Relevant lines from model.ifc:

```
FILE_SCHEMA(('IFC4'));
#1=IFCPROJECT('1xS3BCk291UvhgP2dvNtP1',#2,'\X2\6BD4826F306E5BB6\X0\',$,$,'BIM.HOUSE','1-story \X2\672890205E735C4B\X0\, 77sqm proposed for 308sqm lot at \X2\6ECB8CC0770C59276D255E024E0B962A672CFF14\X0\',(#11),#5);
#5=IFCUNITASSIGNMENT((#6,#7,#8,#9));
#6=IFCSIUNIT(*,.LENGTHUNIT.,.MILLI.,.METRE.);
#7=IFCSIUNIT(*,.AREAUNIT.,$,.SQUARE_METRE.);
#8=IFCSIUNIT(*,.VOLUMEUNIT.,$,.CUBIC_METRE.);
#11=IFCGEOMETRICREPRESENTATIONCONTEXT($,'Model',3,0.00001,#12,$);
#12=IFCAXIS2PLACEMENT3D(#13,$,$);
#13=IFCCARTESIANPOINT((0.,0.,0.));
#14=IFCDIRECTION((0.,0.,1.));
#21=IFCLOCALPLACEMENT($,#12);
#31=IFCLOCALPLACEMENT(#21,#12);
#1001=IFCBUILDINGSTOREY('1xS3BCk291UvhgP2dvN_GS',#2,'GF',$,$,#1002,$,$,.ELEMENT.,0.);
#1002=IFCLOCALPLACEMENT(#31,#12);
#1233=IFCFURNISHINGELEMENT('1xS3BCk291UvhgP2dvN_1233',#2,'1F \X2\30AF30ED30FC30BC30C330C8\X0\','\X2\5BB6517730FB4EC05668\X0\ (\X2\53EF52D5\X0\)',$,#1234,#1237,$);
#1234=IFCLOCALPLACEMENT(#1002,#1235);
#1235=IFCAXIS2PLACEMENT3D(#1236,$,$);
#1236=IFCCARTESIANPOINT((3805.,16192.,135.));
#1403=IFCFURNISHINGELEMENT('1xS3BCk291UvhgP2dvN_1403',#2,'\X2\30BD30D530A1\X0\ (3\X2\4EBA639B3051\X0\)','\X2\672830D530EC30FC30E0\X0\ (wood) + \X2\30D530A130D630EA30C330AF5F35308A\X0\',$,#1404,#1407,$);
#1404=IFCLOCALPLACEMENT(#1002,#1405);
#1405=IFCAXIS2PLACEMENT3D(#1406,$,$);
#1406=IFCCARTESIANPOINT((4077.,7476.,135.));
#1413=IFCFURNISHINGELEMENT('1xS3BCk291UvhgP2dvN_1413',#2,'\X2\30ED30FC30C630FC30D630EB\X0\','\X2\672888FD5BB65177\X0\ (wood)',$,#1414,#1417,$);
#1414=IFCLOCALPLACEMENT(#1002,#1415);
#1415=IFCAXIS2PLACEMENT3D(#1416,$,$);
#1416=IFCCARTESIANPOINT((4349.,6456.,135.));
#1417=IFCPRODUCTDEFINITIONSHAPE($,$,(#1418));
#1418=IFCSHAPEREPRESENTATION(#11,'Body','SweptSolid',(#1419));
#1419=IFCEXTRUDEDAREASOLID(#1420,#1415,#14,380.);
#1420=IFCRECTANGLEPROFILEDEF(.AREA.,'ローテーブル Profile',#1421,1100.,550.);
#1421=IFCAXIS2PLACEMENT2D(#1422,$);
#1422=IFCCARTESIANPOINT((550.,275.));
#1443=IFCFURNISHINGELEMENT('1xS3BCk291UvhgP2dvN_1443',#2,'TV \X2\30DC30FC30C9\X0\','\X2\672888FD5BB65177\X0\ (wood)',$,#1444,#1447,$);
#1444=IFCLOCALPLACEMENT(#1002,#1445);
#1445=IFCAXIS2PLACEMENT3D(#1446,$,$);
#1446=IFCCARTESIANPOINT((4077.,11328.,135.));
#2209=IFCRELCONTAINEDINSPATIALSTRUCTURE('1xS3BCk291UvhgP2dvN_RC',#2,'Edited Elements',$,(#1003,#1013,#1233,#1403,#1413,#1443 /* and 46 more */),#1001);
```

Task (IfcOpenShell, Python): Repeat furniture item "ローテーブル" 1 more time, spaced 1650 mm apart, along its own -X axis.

```python
import ifcopenshell
import ifcopenshell.api.geometry
import ifcopenshell.api.root
import ifcopenshell.util.element
import ifcopenshell.util.placement
import ifcopenshell.util.unit

model = ifcopenshell.open("model.ifc")
unit_scale = ifcopenshell.util.unit.calculate_unit_scale(model)


def reuse_history(source, copy):
    """copy_class also copies each property set's owner history, people and application; keep the originals."""
    for rel in copy.IsDefinedBy:
        if rel.is_a("IfcRelDefinesByProperties") and (history := rel.RelatingPropertyDefinition.OwnerHistory):
            rel.RelatingPropertyDefinition.OwnerHistory = source.OwnerHistory
            ifcopenshell.util.element.remove_deep2(model, history)


source = model.by_id(1413)
base = ifcopenshell.util.placement.get_local_placement(source.ObjectPlacement)
step = -base[:3, 0] * 1.65 / unit_scale

for i in range(1, 2):
    copy = ifcopenshell.api.root.copy_class(model, product=source)
    copy.Representation = ifcopenshell.util.element.copy_deep(
        model, source.Representation, exclude=["IfcGeometricRepresentationContext", "IfcRepresentationMap"]
    )
    reuse_history(source, copy)
    matrix = base.copy()
    matrix[:3, 3] += i * step
    print("added at", matrix[:3, 3].round(3) + 0.0)
    ifcopenshell.api.geometry.edit_object_placement(model, product=copy, matrix=matrix, is_si=False)

model.write("model_edited.ifc")
```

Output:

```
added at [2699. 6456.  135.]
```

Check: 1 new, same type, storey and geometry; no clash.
